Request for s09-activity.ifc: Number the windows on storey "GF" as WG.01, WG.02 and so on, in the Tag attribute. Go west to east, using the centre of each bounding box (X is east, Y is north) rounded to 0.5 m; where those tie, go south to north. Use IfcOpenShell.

First a look at what the model holds.

```python
import ifcopenshell
import ifcopenshell.util.element
import ifcopenshell.util.placement

model = ifcopenshell.open("s09-activity.ifc")
print(model.schema)
storey = next(s for s in model.by_type("IfcBuildingStorey") if s.Name == "GF")
windows = [e for e in ifcopenshell.util.element.get_decomposition(storey) if e.is_a("IfcWindow")]
for e in sorted(windows, key=lambda e: e.id()):
    origin = ifcopenshell.util.placement.get_local_placement(e.ObjectPlacement)[:3, 3]
    print(e.id(), e.Tag, e.Name, origin.round(2) + 0.0, sep=" | ")
```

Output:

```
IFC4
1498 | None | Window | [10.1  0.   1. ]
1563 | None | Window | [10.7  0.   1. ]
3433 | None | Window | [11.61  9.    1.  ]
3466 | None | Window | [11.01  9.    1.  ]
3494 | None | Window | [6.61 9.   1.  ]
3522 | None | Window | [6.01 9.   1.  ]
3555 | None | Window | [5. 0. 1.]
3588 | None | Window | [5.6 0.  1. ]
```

```python
import ifcopenshell
import ifcopenshell.geom
import ifcopenshell.util.element
import ifcopenshell.util.shape

model = ifcopenshell.open("s09-activity.ifc")
settings = ifcopenshell.geom.settings()
settings.set("use-world-coords", True)


def centre(element):
    shape = ifcopenshell.geom.create_shape(settings, element)
    return ifcopenshell.util.shape.get_bbox_centroid(shape.geometry)


storey = next(s for s in model.by_type("IfcBuildingStorey") if s.Name == "GF")
windows = [e for e in ifcopenshell.util.element.get_decomposition(storey) if e.is_a("IfcWindow")]

# Insertion points can sit at a corner or the storey origin, so sort by the geometry (in metres).
centres = {e: centre(e) for e in windows}
windows.sort(key=lambda e: (round(centres[e][0] / 0.5), centres[e][1]))

for i, e in enumerate(windows, start=1):
    number = f"WG.{i:02d}"
    e.Tag = number
    print(e.id(), number)

model.write("s09-activity-out.ifc")
```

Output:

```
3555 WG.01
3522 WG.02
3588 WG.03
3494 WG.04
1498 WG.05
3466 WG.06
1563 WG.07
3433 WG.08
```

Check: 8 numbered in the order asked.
